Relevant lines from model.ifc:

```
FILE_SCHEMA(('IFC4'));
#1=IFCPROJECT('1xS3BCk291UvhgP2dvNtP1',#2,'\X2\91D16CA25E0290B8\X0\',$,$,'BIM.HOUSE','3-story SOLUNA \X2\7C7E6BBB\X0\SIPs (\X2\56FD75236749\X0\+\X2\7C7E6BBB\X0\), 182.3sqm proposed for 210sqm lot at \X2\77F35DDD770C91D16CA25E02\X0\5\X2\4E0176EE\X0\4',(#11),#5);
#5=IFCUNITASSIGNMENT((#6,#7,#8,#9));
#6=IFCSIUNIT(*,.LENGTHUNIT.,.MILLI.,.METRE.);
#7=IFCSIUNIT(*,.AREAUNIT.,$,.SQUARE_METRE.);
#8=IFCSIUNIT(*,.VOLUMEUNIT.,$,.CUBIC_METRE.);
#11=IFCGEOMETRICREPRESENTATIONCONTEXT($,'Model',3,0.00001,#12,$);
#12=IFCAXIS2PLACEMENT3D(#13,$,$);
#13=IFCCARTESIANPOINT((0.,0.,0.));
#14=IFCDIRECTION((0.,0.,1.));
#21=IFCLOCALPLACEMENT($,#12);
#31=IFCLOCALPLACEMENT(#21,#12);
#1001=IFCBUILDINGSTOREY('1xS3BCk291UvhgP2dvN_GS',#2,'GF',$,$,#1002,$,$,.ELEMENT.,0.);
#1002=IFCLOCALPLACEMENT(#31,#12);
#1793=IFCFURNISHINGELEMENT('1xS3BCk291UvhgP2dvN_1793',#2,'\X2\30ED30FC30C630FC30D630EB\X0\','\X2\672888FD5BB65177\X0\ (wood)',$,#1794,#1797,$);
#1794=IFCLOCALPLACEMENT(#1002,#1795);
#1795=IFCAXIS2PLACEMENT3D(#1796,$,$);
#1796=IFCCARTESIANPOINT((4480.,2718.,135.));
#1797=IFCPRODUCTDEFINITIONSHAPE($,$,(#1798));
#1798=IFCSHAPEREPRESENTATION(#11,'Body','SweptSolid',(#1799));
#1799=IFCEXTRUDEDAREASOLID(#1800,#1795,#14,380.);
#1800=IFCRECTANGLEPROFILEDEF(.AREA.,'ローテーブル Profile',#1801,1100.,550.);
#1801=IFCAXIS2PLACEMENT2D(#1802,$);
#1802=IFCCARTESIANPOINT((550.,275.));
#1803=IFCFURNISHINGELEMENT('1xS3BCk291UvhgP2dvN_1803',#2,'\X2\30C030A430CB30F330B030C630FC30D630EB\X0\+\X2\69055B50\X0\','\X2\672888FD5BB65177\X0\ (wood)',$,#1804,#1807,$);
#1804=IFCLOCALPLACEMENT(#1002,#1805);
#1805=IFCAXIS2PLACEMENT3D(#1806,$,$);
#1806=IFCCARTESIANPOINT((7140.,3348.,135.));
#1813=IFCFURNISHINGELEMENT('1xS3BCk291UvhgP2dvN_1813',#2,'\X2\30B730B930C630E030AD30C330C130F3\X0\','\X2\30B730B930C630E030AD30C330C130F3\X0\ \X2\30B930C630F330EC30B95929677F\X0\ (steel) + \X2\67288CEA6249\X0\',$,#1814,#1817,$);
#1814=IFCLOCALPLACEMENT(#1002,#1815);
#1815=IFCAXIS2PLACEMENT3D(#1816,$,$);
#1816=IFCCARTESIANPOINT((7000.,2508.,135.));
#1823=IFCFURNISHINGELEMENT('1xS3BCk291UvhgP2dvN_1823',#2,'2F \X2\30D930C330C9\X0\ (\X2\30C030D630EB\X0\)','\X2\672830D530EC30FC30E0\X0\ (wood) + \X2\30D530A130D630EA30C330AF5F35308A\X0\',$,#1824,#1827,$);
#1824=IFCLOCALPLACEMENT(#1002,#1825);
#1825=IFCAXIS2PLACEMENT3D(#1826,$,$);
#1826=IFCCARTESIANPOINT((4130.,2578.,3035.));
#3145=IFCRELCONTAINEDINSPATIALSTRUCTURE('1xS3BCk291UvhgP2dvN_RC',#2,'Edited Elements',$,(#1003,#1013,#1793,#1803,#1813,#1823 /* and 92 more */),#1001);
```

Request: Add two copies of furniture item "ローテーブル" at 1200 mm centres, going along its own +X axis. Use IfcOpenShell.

```python
import ifcopenshell
import ifcopenshell.api.geometry
import ifcopenshell.api.root
import ifcopenshell.util.element
import ifcopenshell.util.placement
import ifcopenshell.util.unit

model = ifcopenshell.open("model.ifc")
unit_scale = ifcopenshell.util.unit.calculate_unit_scale(model)


def reuse_history(source, copy):
    """copy_class also copies each property set's owner history, people and application; keep the originals."""
    for rel in copy.IsDefinedBy:
        if rel.is_a("IfcRelDefinesByProperties") and (history := rel.RelatingPropertyDefinition.OwnerHistory):
            rel.RelatingPropertyDefinition.OwnerHistory = source.OwnerHistory
            ifcopenshell.util.element.remove_deep2(model, history)


source = model.by_guid("1xS3BCk291UvhgP2dvN_1793")
base = ifcopenshell.util.placement.get_local_placement(source.ObjectPlacement)
step = base[:3, 0] * 1.2 / unit_scale

for i in range(1, 3):
    copy = ifcopenshell.api.root.copy_class(model, product=source)
    copy.Representation = ifcopenshell.util.element.copy_deep(
        model, source.Representation, exclude=["IfcGeometricRepresentationContext", "IfcRepresentationMap"]
    )
    reuse_history(source, copy)
    matrix = base.copy()
    matrix[:3, 3] += i * step
    print("added at", matrix[:3, 3].round(3) + 0.0)
    ifcopenshell.api.geometry.edit_object_placement(model, product=copy, matrix=matrix, is_si=False)

model.write("model_v2.ifc")
```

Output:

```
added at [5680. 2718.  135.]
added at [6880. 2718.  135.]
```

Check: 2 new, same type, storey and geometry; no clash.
